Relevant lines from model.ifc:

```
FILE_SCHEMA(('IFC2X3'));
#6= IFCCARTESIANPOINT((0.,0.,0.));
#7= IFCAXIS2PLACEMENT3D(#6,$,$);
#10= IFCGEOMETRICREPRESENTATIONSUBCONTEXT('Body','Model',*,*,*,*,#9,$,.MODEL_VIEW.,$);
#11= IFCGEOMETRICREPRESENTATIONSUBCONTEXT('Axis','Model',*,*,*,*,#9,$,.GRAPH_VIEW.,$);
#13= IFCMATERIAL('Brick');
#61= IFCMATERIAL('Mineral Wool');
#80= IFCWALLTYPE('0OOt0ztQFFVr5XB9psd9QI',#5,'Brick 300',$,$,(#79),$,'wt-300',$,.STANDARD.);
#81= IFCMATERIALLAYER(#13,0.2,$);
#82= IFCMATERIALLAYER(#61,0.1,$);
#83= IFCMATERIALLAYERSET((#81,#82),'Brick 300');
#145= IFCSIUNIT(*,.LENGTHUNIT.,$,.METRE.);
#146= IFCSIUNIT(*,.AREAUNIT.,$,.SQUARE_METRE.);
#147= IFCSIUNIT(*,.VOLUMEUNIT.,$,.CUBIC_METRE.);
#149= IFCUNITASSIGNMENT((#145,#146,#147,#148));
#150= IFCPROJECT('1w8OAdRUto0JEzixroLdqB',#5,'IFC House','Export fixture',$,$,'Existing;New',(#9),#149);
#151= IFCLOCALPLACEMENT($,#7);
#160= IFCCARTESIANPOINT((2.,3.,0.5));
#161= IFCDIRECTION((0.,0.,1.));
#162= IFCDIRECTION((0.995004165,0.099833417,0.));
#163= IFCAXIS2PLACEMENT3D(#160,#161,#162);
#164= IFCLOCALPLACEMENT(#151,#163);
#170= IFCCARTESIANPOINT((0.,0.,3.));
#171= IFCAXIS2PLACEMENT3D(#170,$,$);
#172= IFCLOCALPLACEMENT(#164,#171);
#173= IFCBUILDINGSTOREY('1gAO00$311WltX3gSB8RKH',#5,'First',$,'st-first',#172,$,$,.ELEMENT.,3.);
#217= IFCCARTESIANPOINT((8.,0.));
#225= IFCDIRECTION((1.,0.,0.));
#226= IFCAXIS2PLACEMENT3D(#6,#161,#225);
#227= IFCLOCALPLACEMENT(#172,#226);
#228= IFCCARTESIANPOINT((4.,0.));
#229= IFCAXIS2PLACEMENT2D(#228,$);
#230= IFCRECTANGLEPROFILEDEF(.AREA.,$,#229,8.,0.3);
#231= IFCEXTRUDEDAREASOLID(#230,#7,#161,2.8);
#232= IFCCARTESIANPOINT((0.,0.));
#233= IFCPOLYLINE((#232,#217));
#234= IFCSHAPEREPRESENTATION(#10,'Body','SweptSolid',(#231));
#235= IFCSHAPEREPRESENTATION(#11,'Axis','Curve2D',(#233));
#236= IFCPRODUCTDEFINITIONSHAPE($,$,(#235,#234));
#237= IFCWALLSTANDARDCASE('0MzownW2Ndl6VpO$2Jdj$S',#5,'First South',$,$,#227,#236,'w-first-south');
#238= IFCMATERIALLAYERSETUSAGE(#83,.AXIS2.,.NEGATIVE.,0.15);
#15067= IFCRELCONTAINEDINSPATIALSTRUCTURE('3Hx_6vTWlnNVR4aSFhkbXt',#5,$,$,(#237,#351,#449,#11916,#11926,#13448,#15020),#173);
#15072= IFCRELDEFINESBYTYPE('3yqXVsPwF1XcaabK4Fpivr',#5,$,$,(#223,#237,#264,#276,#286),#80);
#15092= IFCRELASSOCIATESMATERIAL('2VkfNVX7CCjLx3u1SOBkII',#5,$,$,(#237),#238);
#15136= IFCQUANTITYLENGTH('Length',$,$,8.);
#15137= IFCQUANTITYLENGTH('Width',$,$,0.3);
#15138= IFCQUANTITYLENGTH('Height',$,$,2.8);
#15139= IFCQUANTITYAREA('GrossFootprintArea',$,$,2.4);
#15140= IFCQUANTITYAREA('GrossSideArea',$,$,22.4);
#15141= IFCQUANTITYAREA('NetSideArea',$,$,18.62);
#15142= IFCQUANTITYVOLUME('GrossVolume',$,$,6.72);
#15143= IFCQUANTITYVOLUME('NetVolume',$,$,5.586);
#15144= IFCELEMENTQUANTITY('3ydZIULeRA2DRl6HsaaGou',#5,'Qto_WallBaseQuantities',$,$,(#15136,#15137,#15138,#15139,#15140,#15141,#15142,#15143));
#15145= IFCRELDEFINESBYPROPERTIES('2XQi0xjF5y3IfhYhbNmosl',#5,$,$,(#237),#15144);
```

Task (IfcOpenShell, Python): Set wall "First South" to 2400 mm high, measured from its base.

```python
import ifcopenshell
import ifcopenshell.api.pset
import ifcopenshell.geom
import ifcopenshell.util.element
import ifcopenshell.util.representation
import ifcopenshell.util.shape
import ifcopenshell.util.unit

model = ifcopenshell.open("model.ifc")
unit_scale = ifcopenshell.util.unit.calculate_unit_scale(model)
area_scale = ifcopenshell.util.unit.calculate_unit_scale(model, "AREAUNIT")
volume_scale = ifcopenshell.util.unit.calculate_unit_scale(model, "VOLUMEUNIT")
settings = ifcopenshell.geom.settings()


def volume(element):
    """Net volume in cubic metres, openings subtracted."""
    shape = ifcopenshell.geom.create_shape(settings, element)
    return ifcopenshell.util.shape.get_volume(shape.geometry)


wall = model.by_guid("0MzownW2Ndl6VpO$2Jdj$S")
before = volume(wall)

body = ifcopenshell.util.representation.get_representation(wall, "Model", "Body")
solid = body.Items[0]
old_height = solid.Depth
solid.Depth = 2.4
after = volume(wall)
thickness = 0.3  # wall thickness in metres

# Update the stored height, areas and volumes.
qto = model.by_id(ifcopenshell.util.element.get_pset(wall, "Qto_WallBaseQuantities", should_inherit=False)["id"])
ifcopenshell.api.pset.edit_qto(model, qto=qto, properties={
    "Height": solid.Depth,
    "GrossSideArea": ifcopenshell.util.element.get_pset(wall, "Qto_WallBaseQuantities", "GrossSideArea") * solid.Depth / old_height,
    "NetSideArea": after / thickness / area_scale,
    "GrossVolume": ifcopenshell.util.element.get_pset(wall, "Qto_WallBaseQuantities", "GrossVolume") * solid.Depth / old_height,
    "NetVolume": after / volume_scale,
})

print(f"height {old_height:g} -> {solid.Depth:g}, volume {before:.3f} -> {after:.3f} m3")

model.write("model_rev.ifc")
```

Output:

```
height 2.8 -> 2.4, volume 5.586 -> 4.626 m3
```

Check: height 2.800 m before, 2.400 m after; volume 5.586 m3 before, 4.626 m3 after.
